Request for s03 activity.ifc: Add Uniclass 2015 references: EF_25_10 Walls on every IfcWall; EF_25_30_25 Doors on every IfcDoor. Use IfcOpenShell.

First a look at what the model holds.

```python
import ifcopenshell

model = ifcopenshell.open("s03 activity.ifc")
print(model.schema)
print("classifications:", [c.Name for c in model.by_type("IfcClassification")])
for ifc_class in ("IfcDoor", "IfcRoof", "IfcStair", "IfcWall", "IfcWindow"):
    print(ifc_class, len(model.by_type(ifc_class)))
```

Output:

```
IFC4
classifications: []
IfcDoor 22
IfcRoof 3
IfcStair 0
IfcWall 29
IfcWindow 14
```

```python
import ifcopenshell
import ifcopenshell.api.classification

model = ifcopenshell.open("s03 activity.ifc")

system = ifcopenshell.api.classification.add_classification(model, classification="Uniclass 2015")

codes = {
    "IfcWall": ("EF_25_10", "Walls"),
    "IfcDoor": ("EF_25_30_25", "Doors"),
}
for ifc_class, (code, name) in codes.items():
    products = model.by_type(ifc_class)
    ifcopenshell.api.classification.add_reference(
        model, products=products, classification=system, identification=code, name=name
    )
    print(code, len(products))

model.write("s03 activity_edited.ifc")
```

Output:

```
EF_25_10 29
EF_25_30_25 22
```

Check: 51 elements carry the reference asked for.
